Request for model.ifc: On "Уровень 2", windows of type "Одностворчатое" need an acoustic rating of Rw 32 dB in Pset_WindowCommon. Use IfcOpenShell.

First a look at what the model holds.

```python
import ifcopenshell
import ifcopenshell.util.element

model = ifcopenshell.open("model.ifc")
print(model.schema)
storey = next(s for s in model.by_type("IfcBuildingStorey") if s.Name == "Уровень 2")
windows = [e for e in ifcopenshell.util.element.get_decomposition(storey) if e.is_a("IfcWindow")]
seen = {}
for e in windows:
    element_type = ifcopenshell.util.element.get_type(e)
    key = (element_type.Name if element_type != e and element_type else None, ifcopenshell.util.element.get_pset(e, "Pset_WindowCommon", "AcousticRating"))
    seen[key] = seen.get(key, 0) + 1
for (name, value), count in sorted(seen.items(), key=str):
    print(count, "x", name, "|", value)
```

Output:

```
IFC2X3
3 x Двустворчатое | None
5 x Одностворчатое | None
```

```python
import ifcopenshell
import ifcopenshell.api.pset
import ifcopenshell.util.element

model = ifcopenshell.open("model.ifc")

storey = next(s for s in model.by_type("IfcBuildingStorey") if s.Name == "Уровень 2")
windows = [e for e in ifcopenshell.util.element.get_decomposition(storey) if e.is_a("IfcWindow")]

count = 0
for e in windows:
    element_type = ifcopenshell.util.element.get_type(e)
    if element_type in (None, e) or element_type.Name != "Одностворчатое":
        continue
    # add_pset returns the element's existing set when there is one.
    pset = ifcopenshell.api.pset.add_pset(model, product=e, name="Pset_WindowCommon")
    ifcopenshell.api.pset.edit_pset(model, pset=pset, properties={"AcousticRating": "Rw 32 dB"})
    count += 1

print(count, "windows updated")

model.write("model_rev.ifc")
```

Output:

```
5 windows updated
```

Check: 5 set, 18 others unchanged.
